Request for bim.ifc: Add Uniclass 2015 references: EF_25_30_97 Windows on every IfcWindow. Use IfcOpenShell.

First a look at what the model holds.

```python
import ifcopenshell

model = ifcopenshell.open("bim.ifc")
print(model.schema)
print("classifications:", [c.Name for c in model.by_type("IfcClassification")])
for ifc_class in ("IfcDoor", "IfcRoof", "IfcStair", "IfcWall", "IfcWindow"):
    print(ifc_class, len(model.by_type(ifc_class)))
```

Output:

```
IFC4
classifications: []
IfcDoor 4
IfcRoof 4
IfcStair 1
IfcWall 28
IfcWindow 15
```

```python
import ifcopenshell
import ifcopenshell.api.classification

model = ifcopenshell.open("bim.ifc")

system = ifcopenshell.api.classification.add_classification(model, classification="Uniclass 2015")

codes = {
    "IfcWindow": ("EF_25_30_97", "Windows"),
}
for ifc_class, (code, name) in codes.items():
    products = model.by_type(ifc_class)
    ifcopenshell.api.classification.add_reference(
        model, products=products, classification=system, identification=code, name=name
    )
    print(code, len(products))

model.write("bim_rev.ifc")
```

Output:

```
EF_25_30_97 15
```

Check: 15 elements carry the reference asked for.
